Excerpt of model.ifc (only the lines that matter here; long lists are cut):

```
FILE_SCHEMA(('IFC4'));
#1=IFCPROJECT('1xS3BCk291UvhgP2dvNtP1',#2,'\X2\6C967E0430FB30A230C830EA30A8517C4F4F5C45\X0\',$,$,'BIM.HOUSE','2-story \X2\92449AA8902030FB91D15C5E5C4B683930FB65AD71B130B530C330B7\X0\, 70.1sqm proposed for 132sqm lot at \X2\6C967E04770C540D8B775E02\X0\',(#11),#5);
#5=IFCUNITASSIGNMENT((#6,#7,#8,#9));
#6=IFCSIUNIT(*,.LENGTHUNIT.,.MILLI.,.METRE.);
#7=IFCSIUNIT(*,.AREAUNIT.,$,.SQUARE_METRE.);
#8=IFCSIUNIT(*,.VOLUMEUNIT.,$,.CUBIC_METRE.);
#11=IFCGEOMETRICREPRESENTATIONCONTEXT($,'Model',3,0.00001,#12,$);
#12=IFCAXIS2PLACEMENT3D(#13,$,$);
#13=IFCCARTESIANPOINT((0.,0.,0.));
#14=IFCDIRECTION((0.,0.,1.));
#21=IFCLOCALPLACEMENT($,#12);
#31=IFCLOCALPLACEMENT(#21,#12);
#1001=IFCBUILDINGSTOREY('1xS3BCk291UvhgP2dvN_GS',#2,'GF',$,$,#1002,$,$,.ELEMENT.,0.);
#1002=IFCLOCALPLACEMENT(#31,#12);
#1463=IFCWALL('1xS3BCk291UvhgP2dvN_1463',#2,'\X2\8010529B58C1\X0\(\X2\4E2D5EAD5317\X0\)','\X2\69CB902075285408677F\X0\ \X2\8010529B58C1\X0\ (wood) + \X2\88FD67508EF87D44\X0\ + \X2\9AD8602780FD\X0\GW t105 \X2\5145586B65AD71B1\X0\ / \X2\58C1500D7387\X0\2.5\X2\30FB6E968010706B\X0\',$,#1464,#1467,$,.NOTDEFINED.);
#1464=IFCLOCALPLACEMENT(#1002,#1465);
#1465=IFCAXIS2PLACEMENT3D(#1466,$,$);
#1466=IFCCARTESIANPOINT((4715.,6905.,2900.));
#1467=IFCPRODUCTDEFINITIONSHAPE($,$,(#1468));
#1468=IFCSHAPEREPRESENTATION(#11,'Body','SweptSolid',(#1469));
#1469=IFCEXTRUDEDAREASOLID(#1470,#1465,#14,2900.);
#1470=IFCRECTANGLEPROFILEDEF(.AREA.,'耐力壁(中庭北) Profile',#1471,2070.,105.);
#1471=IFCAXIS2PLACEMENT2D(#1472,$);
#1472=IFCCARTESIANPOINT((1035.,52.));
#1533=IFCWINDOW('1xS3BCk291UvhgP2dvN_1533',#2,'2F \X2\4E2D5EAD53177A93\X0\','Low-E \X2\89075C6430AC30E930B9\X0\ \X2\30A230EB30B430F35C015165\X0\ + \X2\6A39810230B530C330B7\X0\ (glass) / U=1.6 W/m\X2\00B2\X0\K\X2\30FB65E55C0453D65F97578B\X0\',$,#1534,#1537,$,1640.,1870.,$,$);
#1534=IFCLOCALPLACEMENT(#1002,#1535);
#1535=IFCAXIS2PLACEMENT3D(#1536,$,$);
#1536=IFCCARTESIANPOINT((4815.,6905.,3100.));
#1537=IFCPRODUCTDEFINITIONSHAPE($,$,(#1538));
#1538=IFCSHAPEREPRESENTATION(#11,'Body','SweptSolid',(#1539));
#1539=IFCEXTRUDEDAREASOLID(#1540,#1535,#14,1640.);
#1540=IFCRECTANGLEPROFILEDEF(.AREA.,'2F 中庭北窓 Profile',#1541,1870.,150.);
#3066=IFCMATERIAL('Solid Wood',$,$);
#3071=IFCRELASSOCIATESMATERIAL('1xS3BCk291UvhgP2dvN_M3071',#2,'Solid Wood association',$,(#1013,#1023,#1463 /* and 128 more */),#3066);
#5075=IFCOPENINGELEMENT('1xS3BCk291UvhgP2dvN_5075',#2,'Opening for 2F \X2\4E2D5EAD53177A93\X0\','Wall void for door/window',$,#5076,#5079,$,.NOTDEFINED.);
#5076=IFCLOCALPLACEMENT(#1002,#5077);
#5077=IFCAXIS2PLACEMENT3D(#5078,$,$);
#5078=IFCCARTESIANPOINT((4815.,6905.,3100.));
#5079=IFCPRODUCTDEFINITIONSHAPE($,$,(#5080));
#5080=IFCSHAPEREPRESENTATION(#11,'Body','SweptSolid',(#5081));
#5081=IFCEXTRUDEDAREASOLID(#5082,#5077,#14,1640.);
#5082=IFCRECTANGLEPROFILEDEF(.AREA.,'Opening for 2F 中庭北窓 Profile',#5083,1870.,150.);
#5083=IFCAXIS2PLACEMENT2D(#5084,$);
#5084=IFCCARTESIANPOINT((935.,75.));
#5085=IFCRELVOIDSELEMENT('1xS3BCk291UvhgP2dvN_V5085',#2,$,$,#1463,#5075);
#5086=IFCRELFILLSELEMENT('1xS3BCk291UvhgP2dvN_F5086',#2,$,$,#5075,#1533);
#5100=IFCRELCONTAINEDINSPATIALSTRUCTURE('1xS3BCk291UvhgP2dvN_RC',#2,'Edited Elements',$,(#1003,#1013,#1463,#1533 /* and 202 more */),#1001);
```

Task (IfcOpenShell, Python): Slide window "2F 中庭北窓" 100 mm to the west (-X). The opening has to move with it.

```python
import ifcopenshell
import ifcopenshell.api.geometry
import ifcopenshell.util.placement
import ifcopenshell.util.unit

model = ifcopenshell.open("model.ifc")
unit_scale = ifcopenshell.util.unit.calculate_unit_scale(model)

window = model.by_id(1533)
opening = window.FillsVoids[0].RelatingOpeningElement
wall = opening.VoidsElements[0].RelatingBuildingElement

wall_matrix = ifcopenshell.util.placement.get_local_placement(wall.ObjectPlacement)
shift = wall_matrix[:3, 0] * -0.1 / unit_scale
before = ifcopenshell.util.placement.get_local_placement(window.ObjectPlacement)[:3, 3].copy()

# The window is not placed relative to its opening, so move both.
for product in (opening, window):
    matrix = ifcopenshell.util.placement.get_local_placement(product.ObjectPlacement)
    matrix[:3, 3] += shift
    ifcopenshell.api.geometry.edit_object_placement(model, product=product, matrix=matrix, is_si=False)

after = ifcopenshell.util.placement.get_local_placement(window.ObjectPlacement)[:3, 3]
print("window moved by", (after - before).round(3) + 0.0)

model.write("model_updated.ifc")
```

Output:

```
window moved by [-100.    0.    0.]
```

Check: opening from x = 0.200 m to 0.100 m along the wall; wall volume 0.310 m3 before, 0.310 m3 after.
